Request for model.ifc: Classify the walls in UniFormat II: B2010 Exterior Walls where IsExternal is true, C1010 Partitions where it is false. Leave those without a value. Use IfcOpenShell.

First a look at what the model holds.

```python
import ifcopenshell
import ifcopenshell.util.element

model = ifcopenshell.open("model.ifc")
print(model.schema)
print("classifications:", [c.Name for c in model.by_type("IfcClassification")])
values = [ifcopenshell.util.element.get_pset(e, "Pset_WallCommon", "IsExternal") for e in model.by_type("IfcWall")]
for value in (True, False, None):
    print("IsExternal", value, values.count(value))
```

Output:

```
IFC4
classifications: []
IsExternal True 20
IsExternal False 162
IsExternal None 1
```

```python
import ifcopenshell
import ifcopenshell.api.classification
import ifcopenshell.util.element

model = ifcopenshell.open("model.ifc")

system = ifcopenshell.api.classification.add_classification(model, classification="UniFormat II")

walls = model.by_type("IfcWall")
external = {e: ifcopenshell.util.element.get_pset(e, "Pset_WallCommon", "IsExternal") for e in walls}
for flag, code, name in ((True, "B2010", "Exterior Walls"), (False, "C1010", "Partitions")):
    products = [e for e in walls if external[e] is flag]
    ifcopenshell.api.classification.add_reference(
        model, products=products, classification=system, identification=code, name=name
    )
    print(code, len(products))

model.write("model_edited.ifc")
```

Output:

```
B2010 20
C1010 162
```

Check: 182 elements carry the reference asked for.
